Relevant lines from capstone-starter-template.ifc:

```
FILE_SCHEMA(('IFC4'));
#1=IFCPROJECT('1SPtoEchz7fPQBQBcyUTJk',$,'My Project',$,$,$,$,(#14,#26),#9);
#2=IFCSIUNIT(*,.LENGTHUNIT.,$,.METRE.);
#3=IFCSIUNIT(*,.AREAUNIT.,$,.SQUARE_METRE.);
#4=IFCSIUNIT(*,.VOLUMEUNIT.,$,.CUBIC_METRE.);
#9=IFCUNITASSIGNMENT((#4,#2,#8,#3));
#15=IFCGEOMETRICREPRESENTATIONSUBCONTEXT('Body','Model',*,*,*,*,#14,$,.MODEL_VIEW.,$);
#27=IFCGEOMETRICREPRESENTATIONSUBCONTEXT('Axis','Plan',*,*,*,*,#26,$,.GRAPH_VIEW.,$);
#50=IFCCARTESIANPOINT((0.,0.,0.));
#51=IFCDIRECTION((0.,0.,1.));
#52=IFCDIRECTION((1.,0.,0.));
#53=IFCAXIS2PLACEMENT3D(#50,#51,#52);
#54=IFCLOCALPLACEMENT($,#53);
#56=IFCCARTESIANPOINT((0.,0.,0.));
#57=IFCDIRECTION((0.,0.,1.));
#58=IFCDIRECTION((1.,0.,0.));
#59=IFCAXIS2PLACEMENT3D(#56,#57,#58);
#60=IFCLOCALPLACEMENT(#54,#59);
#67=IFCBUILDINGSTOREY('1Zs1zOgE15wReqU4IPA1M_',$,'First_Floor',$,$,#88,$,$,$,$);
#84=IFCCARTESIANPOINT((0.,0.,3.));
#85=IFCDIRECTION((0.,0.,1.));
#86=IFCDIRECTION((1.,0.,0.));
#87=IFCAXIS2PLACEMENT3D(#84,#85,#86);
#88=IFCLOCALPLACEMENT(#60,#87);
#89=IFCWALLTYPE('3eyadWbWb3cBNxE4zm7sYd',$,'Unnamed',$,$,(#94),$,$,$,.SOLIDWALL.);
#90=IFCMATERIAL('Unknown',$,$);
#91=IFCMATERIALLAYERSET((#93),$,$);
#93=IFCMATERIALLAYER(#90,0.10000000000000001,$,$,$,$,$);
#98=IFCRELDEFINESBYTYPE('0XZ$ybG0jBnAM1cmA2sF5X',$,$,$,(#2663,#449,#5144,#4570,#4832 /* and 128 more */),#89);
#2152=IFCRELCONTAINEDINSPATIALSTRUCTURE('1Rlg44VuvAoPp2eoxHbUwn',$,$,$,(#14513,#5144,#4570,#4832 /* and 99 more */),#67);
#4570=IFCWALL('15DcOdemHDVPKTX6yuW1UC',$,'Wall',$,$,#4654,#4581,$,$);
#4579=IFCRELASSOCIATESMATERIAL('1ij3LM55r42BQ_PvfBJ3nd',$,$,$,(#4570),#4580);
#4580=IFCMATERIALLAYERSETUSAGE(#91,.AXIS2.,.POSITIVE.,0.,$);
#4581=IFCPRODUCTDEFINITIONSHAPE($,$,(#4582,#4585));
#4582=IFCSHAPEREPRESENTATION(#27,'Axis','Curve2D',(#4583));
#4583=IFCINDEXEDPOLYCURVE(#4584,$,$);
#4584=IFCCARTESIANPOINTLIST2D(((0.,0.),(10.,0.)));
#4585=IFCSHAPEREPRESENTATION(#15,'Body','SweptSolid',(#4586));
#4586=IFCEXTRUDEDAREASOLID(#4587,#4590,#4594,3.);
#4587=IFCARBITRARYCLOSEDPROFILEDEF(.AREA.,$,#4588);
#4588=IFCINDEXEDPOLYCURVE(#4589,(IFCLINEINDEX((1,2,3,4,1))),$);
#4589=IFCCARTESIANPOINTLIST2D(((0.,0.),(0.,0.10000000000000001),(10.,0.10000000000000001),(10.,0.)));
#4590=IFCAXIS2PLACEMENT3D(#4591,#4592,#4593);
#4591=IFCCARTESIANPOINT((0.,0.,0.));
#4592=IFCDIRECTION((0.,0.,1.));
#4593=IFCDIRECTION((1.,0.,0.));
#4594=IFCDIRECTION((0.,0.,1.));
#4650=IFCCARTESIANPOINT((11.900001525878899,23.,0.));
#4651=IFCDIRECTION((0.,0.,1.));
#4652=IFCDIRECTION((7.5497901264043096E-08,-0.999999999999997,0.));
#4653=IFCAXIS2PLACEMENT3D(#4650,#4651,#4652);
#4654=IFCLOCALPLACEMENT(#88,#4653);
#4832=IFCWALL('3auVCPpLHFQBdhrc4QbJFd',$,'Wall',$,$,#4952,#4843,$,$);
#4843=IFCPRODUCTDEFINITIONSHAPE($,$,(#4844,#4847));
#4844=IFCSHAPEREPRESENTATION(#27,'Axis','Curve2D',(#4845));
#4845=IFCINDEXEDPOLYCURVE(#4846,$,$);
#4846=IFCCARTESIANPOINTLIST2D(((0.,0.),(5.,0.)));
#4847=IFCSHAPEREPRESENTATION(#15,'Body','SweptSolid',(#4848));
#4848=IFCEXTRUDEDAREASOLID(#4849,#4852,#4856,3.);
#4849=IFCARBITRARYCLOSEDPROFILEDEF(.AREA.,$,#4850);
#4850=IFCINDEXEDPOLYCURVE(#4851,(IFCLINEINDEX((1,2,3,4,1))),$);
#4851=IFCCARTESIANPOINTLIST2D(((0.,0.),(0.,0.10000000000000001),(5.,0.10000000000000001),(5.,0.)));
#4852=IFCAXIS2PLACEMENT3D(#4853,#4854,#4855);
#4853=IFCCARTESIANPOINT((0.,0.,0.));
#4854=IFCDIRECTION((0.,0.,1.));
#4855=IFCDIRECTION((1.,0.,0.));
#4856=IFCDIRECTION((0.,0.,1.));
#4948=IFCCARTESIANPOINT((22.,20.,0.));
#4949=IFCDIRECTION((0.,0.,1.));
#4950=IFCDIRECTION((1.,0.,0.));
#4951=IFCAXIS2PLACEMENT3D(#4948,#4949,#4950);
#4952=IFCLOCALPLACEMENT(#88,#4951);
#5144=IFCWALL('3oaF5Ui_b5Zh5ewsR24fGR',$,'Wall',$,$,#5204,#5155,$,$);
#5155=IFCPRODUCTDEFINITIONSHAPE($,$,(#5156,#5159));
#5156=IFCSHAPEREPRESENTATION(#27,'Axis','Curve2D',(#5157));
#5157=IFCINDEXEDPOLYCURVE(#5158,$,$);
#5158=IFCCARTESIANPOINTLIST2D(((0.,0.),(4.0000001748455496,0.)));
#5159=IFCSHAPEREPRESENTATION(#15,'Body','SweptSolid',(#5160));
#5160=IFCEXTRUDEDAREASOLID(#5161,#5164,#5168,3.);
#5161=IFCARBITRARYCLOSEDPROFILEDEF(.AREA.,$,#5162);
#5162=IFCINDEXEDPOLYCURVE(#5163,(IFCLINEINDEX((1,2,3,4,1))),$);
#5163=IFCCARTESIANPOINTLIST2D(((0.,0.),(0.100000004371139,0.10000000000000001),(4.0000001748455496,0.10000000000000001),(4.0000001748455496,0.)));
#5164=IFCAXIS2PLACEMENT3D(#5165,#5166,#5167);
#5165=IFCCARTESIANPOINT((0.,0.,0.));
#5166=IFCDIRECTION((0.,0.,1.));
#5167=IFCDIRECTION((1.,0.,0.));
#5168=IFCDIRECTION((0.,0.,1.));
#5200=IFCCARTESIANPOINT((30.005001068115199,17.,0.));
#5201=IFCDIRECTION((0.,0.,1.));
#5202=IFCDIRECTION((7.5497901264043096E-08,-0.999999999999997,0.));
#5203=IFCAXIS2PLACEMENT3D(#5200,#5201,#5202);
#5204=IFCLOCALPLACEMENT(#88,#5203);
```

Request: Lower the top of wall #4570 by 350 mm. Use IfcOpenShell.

```python
import ifcopenshell
import ifcopenshell.geom
import ifcopenshell.util.representation
import ifcopenshell.util.shape

model = ifcopenshell.open("capstone-starter-template.ifc")
settings = ifcopenshell.geom.settings()


def volume(element):
    """Net volume in cubic metres, openings subtracted."""
    shape = ifcopenshell.geom.create_shape(settings, element)
    return ifcopenshell.util.shape.get_volume(shape.geometry)


wall = model.by_guid("15DcOdemHDVPKTX6yuW1UC")
before = volume(wall)

body = ifcopenshell.util.representation.get_representation(wall, "Model", "Body")
solid = body.Items[0]
old_height = solid.Depth
solid.Depth -= 0.35
after = volume(wall)

print(f"height {old_height:g} -> {solid.Depth:g}, volume {before:.3f} -> {after:.3f} m3")

model.write("capstone-starter-template_rev.ifc")
```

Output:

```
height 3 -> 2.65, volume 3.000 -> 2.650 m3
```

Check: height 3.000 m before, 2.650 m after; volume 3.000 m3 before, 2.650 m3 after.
